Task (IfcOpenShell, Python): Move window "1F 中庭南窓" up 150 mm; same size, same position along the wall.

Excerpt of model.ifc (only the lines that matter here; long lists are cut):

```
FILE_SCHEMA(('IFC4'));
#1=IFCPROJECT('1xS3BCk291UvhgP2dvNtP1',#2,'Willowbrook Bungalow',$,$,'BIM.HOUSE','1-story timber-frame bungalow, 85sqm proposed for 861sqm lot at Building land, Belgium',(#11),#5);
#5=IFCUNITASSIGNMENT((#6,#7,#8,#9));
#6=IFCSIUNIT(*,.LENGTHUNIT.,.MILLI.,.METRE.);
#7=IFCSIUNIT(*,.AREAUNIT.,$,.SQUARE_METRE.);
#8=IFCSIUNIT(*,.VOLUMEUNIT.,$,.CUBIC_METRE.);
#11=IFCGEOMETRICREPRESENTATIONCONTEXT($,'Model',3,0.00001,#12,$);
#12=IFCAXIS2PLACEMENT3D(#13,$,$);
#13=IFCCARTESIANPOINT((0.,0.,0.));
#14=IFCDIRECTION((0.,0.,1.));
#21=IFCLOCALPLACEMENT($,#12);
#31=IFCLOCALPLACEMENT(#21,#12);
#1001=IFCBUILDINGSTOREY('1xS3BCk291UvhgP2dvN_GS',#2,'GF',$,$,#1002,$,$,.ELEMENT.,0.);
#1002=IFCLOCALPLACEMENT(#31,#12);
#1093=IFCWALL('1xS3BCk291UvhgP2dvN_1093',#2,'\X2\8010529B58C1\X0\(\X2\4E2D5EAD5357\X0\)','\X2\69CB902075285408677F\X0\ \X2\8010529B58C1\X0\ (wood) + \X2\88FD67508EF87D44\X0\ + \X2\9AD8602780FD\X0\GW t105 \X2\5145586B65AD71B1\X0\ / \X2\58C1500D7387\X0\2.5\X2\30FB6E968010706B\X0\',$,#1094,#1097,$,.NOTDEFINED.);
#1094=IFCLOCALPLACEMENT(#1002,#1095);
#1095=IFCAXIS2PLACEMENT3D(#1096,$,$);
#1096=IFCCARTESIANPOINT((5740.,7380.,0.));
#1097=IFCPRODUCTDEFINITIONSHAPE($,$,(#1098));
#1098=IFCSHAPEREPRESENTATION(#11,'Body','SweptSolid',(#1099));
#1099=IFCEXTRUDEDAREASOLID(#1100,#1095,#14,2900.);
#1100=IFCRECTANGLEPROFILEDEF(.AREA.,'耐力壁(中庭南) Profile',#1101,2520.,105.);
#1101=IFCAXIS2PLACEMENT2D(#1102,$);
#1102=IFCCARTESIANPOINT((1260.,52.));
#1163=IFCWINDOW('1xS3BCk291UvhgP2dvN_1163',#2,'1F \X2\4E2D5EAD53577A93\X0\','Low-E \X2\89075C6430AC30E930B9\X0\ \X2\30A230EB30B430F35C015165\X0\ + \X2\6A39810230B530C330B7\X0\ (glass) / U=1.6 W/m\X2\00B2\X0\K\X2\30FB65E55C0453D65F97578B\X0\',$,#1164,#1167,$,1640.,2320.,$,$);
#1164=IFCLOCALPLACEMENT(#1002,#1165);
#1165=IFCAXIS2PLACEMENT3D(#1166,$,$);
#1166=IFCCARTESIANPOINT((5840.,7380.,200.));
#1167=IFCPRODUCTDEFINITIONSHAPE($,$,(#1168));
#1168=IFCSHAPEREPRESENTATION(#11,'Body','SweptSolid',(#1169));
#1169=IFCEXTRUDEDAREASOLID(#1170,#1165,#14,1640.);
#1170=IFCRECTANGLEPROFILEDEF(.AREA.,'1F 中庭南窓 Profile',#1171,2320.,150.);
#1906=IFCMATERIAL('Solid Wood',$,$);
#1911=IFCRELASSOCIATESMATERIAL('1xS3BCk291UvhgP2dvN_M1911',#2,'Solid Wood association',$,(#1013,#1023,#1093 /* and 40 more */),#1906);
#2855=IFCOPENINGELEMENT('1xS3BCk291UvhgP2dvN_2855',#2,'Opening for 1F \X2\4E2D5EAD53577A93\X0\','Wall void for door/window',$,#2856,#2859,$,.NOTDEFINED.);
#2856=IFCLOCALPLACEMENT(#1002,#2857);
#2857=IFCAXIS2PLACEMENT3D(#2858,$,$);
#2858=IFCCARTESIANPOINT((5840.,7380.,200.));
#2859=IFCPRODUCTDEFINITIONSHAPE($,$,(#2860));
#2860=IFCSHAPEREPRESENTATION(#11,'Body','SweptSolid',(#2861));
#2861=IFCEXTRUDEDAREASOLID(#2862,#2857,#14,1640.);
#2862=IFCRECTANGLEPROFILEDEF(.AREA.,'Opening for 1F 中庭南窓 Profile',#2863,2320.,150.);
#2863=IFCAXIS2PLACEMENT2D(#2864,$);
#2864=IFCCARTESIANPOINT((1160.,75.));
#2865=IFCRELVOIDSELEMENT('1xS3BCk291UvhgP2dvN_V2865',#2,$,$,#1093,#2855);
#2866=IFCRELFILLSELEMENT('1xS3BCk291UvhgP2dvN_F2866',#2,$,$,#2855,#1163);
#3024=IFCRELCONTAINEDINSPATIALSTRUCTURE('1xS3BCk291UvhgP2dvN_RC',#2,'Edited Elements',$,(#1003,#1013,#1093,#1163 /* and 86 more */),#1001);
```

```python
import numpy as np
import ifcopenshell
import ifcopenshell.api.geometry
import ifcopenshell.util.placement
import ifcopenshell.util.unit

model = ifcopenshell.open("model.ifc")
unit_scale = ifcopenshell.util.unit.calculate_unit_scale(model)

window = model.by_guid("1xS3BCk291UvhgP2dvN_1163")
opening = window.FillsVoids[0].RelatingOpeningElement
dz = 0.15 / unit_scale

shift = np.array([0.0, 0.0, dz])
# The window is not placed relative to its opening, so move both.
for product in (opening, window):
    matrix = ifcopenshell.util.placement.get_local_placement(product.ObjectPlacement)
    matrix[:3, 3] += shift
    ifcopenshell.api.geometry.edit_object_placement(model, product=product, matrix=matrix, is_si=False)

print(f"moved by {dz * unit_scale:+.3f} m")

model.write("model_rev.ifc")
```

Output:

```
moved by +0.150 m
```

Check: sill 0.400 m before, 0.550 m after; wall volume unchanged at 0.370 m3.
